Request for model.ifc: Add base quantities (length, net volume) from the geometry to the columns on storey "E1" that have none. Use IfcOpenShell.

First a look at what the model holds.

```python
import ifcopenshell
import ifcopenshell.util.element
import ifcopenshell.util.unit

model = ifcopenshell.open("model.ifc")
print(model.schema)
for unit_type in ("LENGTHUNIT", "AREAUNIT", "VOLUMEUNIT"):
    print(unit_type, ifcopenshell.util.unit.calculate_unit_scale(model, unit_type))
storey = next(s for s in model.by_type("IfcBuildingStorey") if s.Name == "E1")
columns = [e for e in ifcopenshell.util.element.get_decomposition(storey) if e.is_a("IfcColumn")]
for e in sorted(columns, key=lambda e: e.id()):
    print(e.id(), e.is_a(), e.Name, list(ifcopenshell.util.element.get_psets(e, qtos_only=True)), sep=" | ")
```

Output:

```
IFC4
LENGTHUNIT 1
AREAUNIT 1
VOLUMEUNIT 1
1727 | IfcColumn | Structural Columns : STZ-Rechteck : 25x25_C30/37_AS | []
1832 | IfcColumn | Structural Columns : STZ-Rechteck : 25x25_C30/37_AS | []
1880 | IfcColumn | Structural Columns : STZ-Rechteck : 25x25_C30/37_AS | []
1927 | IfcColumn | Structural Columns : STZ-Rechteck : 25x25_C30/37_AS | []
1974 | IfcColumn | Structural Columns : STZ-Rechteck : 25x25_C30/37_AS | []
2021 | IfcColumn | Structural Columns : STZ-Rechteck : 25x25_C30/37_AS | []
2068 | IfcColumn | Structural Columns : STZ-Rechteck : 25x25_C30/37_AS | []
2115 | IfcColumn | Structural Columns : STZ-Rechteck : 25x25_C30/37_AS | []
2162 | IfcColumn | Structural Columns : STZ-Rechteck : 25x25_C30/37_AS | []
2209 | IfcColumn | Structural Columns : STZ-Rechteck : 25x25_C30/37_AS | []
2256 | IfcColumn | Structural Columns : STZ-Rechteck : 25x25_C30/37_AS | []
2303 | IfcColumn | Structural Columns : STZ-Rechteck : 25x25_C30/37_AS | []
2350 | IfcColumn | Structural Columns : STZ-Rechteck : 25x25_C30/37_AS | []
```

```python
import ifcopenshell
import ifcopenshell.api.pset
import ifcopenshell.geom
import ifcopenshell.util.element
import ifcopenshell.util.shape
import ifcopenshell.util.unit

model = ifcopenshell.open("model.ifc")
unit_scale = ifcopenshell.util.unit.calculate_unit_scale(model)
volume_scale = ifcopenshell.util.unit.calculate_unit_scale(model, "VOLUMEUNIT")
settings = ifcopenshell.geom.settings()

storey = next(s for s in model.by_type("IfcBuildingStorey") if s.Name == "E1")
columns = [e for e in ifcopenshell.util.element.get_decomposition(storey) if e.is_a("IfcColumn")]

for e in sorted(columns, key=lambda e: e.id()):
    if ifcopenshell.util.element.get_psets(e, qtos_only=True, should_inherit=False):
        continue
    # Geometry comes back in metres, in the element's own axes.
    shape = ifcopenshell.geom.create_shape(settings, e)
    values = {
        "Length": ifcopenshell.util.shape.get_z(shape.geometry) / unit_scale,
        "NetVolume": ifcopenshell.util.shape.get_volume(shape.geometry) / volume_scale,
    }
    qto = ifcopenshell.api.pset.add_qto(model, product=e, name="Qto_ColumnBaseQuantities")
    ifcopenshell.api.pset.edit_qto(model, qto=qto, properties=values)
    print(e.id(), {k: round(v, 3) for k, v in values.items()})

model.write("model_rev.ifc")
```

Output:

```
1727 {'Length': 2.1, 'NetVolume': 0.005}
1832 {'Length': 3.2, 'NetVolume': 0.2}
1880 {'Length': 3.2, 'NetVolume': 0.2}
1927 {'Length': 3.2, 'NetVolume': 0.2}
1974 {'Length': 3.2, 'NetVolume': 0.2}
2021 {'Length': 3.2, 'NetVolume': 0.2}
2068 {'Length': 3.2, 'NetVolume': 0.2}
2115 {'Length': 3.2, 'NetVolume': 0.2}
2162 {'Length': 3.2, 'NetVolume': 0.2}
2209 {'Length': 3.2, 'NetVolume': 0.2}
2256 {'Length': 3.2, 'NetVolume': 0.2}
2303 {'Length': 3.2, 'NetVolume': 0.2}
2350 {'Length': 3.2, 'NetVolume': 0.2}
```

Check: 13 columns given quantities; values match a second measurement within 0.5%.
